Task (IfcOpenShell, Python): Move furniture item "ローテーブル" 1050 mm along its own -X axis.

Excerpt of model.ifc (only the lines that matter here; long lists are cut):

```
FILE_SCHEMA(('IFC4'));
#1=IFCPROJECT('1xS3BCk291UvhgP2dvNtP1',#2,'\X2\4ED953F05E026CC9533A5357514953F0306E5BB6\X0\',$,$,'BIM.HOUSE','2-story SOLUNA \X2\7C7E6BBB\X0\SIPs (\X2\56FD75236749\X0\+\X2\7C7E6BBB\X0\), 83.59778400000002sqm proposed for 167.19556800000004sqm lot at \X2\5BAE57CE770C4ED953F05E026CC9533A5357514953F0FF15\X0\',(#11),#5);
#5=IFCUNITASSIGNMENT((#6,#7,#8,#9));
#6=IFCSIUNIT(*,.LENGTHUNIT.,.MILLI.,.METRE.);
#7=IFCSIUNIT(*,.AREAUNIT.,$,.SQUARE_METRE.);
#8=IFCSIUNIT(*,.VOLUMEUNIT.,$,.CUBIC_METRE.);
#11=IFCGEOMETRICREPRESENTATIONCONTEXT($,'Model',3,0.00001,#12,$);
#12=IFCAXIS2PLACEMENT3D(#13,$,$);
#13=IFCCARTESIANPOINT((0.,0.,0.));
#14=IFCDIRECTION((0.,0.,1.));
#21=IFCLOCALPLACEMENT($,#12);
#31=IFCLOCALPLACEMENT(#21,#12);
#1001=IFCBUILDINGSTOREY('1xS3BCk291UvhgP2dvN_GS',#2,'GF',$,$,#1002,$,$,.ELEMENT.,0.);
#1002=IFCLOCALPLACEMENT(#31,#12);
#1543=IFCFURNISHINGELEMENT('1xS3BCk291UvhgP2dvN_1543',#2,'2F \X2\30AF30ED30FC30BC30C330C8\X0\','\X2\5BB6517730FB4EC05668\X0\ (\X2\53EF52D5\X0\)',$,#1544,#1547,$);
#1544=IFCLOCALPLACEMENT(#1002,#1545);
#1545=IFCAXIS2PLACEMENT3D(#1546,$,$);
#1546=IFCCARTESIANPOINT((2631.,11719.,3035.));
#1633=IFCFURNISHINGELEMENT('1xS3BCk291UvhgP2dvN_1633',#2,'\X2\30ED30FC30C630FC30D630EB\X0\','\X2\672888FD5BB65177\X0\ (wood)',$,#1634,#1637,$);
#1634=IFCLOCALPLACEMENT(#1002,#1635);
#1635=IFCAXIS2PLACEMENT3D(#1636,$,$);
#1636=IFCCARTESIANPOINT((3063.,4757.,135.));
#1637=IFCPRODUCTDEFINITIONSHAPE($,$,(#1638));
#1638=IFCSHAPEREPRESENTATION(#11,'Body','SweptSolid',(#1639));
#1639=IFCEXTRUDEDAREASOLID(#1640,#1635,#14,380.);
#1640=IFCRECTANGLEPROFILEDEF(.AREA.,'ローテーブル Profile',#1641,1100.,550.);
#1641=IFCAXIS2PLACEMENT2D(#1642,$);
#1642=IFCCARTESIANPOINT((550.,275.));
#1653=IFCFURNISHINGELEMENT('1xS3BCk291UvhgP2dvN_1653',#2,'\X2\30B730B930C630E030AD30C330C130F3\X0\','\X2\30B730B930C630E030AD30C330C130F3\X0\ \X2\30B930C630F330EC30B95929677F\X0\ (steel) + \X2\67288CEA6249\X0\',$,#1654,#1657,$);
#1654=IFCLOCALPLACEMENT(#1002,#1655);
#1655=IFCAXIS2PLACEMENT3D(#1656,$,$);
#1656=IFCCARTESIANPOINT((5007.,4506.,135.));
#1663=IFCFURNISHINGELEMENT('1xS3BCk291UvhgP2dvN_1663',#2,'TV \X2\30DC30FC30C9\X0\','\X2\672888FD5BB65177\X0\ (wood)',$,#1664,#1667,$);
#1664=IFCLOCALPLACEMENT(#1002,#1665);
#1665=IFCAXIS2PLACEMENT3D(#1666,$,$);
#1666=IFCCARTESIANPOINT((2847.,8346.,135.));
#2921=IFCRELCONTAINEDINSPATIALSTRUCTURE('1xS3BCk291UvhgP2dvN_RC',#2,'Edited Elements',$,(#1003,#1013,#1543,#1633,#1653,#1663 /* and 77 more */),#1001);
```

```python
import ifcopenshell
import ifcopenshell.api.geometry
import ifcopenshell.util.placement

model = ifcopenshell.open("model.ifc")

item = model.by_guid("1xS3BCk291UvhgP2dvN_1633")
matrix = ifcopenshell.util.placement.get_local_placement(item.ObjectPlacement)
matrix[:3, 3] -= matrix[:3, 0] * 1050.0
ifcopenshell.api.geometry.edit_object_placement(model, product=item, matrix=matrix, is_si=False)

print(ifcopenshell.util.placement.get_local_placement(item.ObjectPlacement).round(3) + 0.0)

model.write("model_rev.ifc")
```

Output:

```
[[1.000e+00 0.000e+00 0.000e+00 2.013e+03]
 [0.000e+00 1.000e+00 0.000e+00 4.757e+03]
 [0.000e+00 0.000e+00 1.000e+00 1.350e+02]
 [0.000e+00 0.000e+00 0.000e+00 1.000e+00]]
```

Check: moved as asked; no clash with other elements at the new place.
